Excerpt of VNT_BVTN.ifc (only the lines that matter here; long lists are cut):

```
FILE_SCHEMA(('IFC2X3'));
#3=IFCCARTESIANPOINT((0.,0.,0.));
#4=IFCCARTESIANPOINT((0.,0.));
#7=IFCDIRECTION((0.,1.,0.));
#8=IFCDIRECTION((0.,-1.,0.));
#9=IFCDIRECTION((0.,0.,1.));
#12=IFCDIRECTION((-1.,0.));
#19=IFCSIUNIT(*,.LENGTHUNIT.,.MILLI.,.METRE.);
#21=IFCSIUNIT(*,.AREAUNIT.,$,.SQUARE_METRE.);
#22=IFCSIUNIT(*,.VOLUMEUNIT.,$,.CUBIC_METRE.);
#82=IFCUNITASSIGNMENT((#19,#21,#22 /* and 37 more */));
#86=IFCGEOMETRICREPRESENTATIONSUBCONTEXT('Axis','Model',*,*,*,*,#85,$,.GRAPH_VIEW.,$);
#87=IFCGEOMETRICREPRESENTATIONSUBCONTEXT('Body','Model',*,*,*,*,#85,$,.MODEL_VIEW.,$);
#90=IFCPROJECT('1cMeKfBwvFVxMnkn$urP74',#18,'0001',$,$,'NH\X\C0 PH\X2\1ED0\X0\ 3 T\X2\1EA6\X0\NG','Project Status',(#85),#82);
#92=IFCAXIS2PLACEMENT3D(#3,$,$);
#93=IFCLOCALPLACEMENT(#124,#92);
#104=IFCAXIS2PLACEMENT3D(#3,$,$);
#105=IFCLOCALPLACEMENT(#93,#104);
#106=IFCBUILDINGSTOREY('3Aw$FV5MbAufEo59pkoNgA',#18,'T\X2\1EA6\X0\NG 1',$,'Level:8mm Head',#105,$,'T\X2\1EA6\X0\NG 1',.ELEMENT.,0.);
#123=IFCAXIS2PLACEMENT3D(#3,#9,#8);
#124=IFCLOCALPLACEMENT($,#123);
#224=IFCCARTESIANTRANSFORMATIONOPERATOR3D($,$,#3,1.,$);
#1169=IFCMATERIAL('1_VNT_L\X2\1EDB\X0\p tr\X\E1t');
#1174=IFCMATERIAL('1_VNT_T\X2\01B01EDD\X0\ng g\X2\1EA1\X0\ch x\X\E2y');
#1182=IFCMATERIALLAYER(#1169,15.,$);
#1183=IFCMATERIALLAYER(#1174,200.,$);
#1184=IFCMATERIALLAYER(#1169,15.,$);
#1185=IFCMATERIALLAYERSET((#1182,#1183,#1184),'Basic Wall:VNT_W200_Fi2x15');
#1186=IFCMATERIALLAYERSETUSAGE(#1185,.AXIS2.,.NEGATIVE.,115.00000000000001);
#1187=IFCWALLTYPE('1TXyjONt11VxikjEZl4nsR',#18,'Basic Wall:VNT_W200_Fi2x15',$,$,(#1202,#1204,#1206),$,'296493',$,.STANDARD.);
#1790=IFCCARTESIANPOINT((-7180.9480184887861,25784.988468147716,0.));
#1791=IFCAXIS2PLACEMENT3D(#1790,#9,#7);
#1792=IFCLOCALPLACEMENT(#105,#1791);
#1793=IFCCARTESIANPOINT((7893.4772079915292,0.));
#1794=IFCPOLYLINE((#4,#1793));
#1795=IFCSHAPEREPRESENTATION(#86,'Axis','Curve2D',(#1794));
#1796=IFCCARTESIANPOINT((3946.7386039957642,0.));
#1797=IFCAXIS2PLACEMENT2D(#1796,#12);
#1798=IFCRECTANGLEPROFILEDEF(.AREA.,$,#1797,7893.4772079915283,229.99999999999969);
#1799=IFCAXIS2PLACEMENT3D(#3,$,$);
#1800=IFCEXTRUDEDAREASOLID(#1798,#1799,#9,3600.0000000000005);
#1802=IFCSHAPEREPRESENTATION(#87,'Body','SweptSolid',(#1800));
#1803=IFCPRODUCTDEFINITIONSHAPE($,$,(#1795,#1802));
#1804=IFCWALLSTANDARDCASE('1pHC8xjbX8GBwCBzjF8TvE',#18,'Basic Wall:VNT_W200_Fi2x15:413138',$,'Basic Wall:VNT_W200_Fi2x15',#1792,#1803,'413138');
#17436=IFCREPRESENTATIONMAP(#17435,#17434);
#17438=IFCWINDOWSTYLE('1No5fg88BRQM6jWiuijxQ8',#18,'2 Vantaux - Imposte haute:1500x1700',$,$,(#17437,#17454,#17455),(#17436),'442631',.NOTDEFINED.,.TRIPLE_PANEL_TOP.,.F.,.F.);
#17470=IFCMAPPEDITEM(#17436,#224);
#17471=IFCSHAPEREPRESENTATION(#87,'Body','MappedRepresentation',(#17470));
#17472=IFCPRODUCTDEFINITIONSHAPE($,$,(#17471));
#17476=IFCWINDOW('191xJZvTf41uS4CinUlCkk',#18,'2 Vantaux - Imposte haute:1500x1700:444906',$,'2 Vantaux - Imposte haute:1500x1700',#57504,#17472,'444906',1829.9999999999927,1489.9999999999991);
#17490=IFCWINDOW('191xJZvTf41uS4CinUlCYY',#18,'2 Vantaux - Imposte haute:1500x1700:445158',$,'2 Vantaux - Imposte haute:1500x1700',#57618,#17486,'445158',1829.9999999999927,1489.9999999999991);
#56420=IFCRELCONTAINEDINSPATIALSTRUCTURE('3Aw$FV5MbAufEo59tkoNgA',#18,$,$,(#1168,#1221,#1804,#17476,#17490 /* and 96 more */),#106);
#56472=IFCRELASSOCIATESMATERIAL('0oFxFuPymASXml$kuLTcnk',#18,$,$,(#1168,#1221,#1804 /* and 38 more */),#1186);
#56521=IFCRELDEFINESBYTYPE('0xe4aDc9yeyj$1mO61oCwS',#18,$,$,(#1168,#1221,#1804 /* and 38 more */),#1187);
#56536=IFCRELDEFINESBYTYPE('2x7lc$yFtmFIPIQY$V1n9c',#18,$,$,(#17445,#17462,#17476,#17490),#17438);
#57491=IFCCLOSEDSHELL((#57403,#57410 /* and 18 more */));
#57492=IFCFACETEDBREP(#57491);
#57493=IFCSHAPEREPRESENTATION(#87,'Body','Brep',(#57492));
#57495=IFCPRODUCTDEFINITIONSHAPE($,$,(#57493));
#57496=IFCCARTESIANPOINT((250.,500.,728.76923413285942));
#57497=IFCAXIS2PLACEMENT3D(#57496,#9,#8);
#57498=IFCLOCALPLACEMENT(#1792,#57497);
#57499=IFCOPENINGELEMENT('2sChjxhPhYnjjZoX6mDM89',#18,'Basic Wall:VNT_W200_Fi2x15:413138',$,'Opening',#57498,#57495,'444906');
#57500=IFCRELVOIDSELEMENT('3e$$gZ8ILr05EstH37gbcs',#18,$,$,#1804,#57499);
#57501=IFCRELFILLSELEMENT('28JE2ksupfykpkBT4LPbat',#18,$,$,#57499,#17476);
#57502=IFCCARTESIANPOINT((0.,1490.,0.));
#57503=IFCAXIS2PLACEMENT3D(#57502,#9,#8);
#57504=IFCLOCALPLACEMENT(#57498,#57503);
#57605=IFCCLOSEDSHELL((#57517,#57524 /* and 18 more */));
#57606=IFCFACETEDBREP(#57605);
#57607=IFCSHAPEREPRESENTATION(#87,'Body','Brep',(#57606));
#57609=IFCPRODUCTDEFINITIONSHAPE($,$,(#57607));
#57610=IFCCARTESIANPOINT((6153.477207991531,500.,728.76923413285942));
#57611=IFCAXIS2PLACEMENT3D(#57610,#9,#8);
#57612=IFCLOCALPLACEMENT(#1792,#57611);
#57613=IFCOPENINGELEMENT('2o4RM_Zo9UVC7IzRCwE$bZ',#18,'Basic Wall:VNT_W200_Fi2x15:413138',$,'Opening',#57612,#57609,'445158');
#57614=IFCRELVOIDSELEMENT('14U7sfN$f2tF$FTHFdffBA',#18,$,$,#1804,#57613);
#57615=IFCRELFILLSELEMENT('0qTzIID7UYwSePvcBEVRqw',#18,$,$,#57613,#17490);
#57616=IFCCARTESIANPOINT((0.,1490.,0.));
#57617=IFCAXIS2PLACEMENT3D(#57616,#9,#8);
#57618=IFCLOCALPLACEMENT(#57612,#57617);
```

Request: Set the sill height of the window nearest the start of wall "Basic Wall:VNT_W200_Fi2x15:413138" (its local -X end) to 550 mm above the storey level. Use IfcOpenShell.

```python
import numpy as np
import ifcopenshell
import ifcopenshell.api.geometry
import ifcopenshell.geom
import ifcopenshell.util.element
import ifcopenshell.util.placement
import ifcopenshell.util.shape
import ifcopenshell.util.unit

model = ifcopenshell.open("VNT_BVTN.ifc")
unit_scale = ifcopenshell.util.unit.calculate_unit_scale(model)

window = model.by_id(17476)
opening = window.FillsVoids[0].RelatingOpeningElement
storey = ifcopenshell.util.element.get_container(window, ifc_class="IfcBuildingStorey")
level = ifcopenshell.util.placement.get_local_placement(storey.ObjectPlacement)[2, 3]

# The opening's origin need not be at the sill, so measure its lowest point.
shape = ifcopenshell.geom.create_shape(ifcopenshell.geom.settings(), opening)
bottom = ifcopenshell.util.shape.get_shape_bottom_elevation(shape, shape.geometry) / unit_scale
dz = level + 0.55 / unit_scale - bottom

shift = np.array([0.0, 0.0, dz])
# The window is placed relative to its opening, so it follows when the opening moves.
matrix = ifcopenshell.util.placement.get_local_placement(opening.ObjectPlacement)
matrix[:3, 3] += shift
ifcopenshell.api.geometry.edit_object_placement(
    model, product=opening, matrix=matrix, is_si=False, should_transform_children=True
)

print(f"moved by {dz * unit_scale:+.3f} m")

model.write("VNT_BVTN-out.ifc")
```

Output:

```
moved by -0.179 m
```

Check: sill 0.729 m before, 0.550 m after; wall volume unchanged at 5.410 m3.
